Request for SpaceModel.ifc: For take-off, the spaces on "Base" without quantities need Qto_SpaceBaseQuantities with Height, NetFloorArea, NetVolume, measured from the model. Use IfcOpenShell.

First a look at what the model holds.

```python
import ifcopenshell
import ifcopenshell.util.element
import ifcopenshell.util.unit

model = ifcopenshell.open("SpaceModel.ifc")
print(model.schema)
for unit_type in ("LENGTHUNIT", "AREAUNIT", "VOLUMEUNIT"):
    print(unit_type, ifcopenshell.util.unit.calculate_unit_scale(model, unit_type))
storey = next(s for s in model.by_type("IfcBuildingStorey") if s.Name == "Base")
spaces = [e for e in ifcopenshell.util.element.get_decomposition(storey) if e.is_a("IfcSpace")]
for e in sorted(spaces, key=lambda e: e.id()):
    print(e.id(), e.is_a(), e.Name, list(ifcopenshell.util.element.get_psets(e, qtos_only=True)), sep=" | ")
```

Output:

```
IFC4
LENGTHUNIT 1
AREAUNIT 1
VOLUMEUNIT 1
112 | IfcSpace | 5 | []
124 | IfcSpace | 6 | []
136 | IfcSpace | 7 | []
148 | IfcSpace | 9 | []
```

```python
import ifcopenshell
import ifcopenshell.api.pset
import ifcopenshell.geom
import ifcopenshell.util.element
import ifcopenshell.util.shape
import ifcopenshell.util.unit

model = ifcopenshell.open("SpaceModel.ifc")
unit_scale = ifcopenshell.util.unit.calculate_unit_scale(model)
area_scale = ifcopenshell.util.unit.calculate_unit_scale(model, "AREAUNIT")
volume_scale = ifcopenshell.util.unit.calculate_unit_scale(model, "VOLUMEUNIT")
settings = ifcopenshell.geom.settings()

storey = next(s for s in model.by_type("IfcBuildingStorey") if s.Name == "Base")
spaces = [e for e in ifcopenshell.util.element.get_decomposition(storey) if e.is_a("IfcSpace")]

for e in sorted(spaces, key=lambda e: e.id()):
    if ifcopenshell.util.element.get_psets(e, qtos_only=True, should_inherit=False):
        continue
    # Geometry comes back in metres, in the element's own axes.
    shape = ifcopenshell.geom.create_shape(settings, e)
    values = {
        "Height": ifcopenshell.util.shape.get_z(shape.geometry) / unit_scale,
        "NetFloorArea": ifcopenshell.util.shape.get_footprint_area(shape.geometry) / area_scale,
        "NetVolume": ifcopenshell.util.shape.get_volume(shape.geometry) / volume_scale,
    }
    qto = ifcopenshell.api.pset.add_qto(model, product=e, name="Qto_SpaceBaseQuantities")
    ifcopenshell.api.pset.edit_qto(model, qto=qto, properties=values)
    print(e.id(), {k: round(v, 3) for k, v in values.items()})

model.write("SpaceModel_rev.ifc")
```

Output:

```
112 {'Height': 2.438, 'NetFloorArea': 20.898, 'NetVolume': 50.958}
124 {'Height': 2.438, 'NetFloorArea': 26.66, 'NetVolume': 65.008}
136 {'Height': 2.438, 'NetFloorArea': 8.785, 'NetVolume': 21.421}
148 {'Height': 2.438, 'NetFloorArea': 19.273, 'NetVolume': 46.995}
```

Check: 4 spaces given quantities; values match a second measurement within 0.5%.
